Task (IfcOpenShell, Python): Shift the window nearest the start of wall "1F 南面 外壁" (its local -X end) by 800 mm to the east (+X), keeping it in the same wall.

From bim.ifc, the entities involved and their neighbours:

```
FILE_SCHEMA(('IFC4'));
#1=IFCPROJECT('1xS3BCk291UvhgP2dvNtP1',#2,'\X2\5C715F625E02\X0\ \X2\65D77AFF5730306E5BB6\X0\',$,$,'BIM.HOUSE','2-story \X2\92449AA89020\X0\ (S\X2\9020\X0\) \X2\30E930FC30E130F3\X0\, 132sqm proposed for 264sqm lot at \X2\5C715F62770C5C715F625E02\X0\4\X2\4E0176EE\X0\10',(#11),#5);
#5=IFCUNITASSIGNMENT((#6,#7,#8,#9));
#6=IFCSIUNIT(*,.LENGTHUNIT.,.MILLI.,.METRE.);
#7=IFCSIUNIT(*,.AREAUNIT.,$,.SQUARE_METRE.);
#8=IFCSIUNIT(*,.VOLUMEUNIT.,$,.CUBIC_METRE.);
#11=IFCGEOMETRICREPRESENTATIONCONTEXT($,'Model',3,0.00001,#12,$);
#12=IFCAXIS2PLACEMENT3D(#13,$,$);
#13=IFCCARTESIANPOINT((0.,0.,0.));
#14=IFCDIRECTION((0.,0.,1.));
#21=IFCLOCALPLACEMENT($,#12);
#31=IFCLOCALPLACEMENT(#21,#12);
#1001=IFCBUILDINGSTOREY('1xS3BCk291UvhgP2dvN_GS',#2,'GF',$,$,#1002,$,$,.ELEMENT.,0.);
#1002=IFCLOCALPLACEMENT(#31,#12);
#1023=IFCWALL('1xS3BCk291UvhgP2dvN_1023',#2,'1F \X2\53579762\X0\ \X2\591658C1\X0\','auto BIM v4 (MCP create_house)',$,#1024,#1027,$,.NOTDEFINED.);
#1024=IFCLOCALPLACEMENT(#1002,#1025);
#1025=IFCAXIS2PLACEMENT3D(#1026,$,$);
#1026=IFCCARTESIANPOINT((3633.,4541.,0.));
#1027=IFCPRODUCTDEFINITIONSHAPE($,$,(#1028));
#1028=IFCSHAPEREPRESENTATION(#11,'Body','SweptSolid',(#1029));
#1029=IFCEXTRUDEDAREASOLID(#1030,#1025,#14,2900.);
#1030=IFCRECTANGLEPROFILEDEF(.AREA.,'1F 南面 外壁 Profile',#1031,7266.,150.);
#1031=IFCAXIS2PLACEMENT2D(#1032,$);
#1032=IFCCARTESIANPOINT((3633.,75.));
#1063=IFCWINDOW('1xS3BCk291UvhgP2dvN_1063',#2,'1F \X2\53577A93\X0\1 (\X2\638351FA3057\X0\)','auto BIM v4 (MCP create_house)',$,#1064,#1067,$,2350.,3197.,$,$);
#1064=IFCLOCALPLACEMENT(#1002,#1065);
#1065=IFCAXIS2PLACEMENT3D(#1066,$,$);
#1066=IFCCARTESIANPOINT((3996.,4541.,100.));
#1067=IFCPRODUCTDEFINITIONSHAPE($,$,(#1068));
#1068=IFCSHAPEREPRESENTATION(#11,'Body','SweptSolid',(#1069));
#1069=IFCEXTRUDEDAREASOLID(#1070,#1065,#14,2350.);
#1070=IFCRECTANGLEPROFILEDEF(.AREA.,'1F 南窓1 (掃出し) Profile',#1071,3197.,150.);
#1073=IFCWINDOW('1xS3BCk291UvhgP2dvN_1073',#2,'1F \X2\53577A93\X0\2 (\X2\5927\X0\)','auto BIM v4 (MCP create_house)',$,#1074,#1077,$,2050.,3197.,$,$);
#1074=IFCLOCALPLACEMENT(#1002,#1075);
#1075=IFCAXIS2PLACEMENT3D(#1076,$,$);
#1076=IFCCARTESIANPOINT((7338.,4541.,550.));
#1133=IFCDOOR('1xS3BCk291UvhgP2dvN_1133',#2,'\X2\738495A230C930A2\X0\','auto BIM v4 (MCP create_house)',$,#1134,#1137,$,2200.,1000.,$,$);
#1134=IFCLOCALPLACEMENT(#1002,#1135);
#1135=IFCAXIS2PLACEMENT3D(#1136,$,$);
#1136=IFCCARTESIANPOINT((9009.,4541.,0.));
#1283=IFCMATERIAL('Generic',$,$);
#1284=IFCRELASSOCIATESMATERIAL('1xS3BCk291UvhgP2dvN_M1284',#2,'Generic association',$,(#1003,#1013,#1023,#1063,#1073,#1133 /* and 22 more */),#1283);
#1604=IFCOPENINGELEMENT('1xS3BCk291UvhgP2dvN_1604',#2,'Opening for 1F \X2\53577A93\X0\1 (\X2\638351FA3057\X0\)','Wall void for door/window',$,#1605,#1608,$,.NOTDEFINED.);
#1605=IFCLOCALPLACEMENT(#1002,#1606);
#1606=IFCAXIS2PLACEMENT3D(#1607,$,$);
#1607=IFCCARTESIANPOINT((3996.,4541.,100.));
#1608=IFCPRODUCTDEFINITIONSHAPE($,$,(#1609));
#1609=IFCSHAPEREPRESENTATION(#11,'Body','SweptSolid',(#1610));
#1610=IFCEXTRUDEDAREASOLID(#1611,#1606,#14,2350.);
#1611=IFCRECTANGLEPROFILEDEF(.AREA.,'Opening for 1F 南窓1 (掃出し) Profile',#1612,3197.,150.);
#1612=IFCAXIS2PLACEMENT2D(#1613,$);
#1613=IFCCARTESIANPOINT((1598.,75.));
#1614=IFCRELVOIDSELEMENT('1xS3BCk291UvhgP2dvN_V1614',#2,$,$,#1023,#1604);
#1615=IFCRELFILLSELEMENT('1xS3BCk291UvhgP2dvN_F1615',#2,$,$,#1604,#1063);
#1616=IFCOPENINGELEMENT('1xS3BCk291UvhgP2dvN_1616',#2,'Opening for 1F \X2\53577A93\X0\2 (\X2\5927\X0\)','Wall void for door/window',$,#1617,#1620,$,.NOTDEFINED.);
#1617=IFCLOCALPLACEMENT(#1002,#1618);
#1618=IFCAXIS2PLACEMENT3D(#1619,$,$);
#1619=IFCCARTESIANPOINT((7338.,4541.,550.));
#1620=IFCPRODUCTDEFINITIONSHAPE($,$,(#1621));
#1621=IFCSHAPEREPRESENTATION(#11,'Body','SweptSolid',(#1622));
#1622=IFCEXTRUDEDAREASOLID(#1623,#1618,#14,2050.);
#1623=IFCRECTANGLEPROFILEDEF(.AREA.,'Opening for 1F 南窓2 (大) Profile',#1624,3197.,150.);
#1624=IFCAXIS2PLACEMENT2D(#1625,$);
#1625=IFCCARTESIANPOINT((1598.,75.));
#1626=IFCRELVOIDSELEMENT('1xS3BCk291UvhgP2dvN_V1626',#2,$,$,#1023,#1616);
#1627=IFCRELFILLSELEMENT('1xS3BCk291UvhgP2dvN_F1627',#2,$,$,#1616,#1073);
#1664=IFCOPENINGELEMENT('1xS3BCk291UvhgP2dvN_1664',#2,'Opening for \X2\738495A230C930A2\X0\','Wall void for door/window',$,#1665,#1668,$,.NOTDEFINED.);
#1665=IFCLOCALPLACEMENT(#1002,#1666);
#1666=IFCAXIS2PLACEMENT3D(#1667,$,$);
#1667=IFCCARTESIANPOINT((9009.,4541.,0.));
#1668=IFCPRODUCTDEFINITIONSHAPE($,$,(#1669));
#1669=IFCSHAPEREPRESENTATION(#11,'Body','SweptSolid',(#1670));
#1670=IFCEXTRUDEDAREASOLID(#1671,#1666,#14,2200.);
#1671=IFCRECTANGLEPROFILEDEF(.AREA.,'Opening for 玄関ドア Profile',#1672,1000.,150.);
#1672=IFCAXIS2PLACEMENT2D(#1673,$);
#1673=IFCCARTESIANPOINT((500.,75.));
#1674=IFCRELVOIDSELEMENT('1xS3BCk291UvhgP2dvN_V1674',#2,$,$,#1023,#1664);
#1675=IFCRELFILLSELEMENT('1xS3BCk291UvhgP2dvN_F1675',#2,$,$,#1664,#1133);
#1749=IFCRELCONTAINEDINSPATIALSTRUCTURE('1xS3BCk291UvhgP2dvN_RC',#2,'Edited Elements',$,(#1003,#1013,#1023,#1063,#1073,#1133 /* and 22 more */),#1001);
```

```python
import ifcopenshell
import ifcopenshell.api.geometry
import ifcopenshell.util.placement
import ifcopenshell.util.unit

model = ifcopenshell.open("bim.ifc")
unit_scale = ifcopenshell.util.unit.calculate_unit_scale(model)

window = model.by_guid("1xS3BCk291UvhgP2dvN_1063")
opening = window.FillsVoids[0].RelatingOpeningElement
wall = opening.VoidsElements[0].RelatingBuildingElement

wall_matrix = ifcopenshell.util.placement.get_local_placement(wall.ObjectPlacement)
shift = wall_matrix[:3, 0] * 0.8 / unit_scale
before = ifcopenshell.util.placement.get_local_placement(window.ObjectPlacement)[:3, 3].copy()

# The window is not placed relative to its opening, so move both.
for product in (opening, window):
    matrix = ifcopenshell.util.placement.get_local_placement(product.ObjectPlacement)
    matrix[:3, 3] += shift
    ifcopenshell.api.geometry.edit_object_placement(model, product=product, matrix=matrix, is_si=False)

after = ifcopenshell.util.placement.get_local_placement(window.ObjectPlacement)[:3, 3]
print("window moved by", (after - before).round(3) + 0.0)

model.write("bim_updated.ifc")
```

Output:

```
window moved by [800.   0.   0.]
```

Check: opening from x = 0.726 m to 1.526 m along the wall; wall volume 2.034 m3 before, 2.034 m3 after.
